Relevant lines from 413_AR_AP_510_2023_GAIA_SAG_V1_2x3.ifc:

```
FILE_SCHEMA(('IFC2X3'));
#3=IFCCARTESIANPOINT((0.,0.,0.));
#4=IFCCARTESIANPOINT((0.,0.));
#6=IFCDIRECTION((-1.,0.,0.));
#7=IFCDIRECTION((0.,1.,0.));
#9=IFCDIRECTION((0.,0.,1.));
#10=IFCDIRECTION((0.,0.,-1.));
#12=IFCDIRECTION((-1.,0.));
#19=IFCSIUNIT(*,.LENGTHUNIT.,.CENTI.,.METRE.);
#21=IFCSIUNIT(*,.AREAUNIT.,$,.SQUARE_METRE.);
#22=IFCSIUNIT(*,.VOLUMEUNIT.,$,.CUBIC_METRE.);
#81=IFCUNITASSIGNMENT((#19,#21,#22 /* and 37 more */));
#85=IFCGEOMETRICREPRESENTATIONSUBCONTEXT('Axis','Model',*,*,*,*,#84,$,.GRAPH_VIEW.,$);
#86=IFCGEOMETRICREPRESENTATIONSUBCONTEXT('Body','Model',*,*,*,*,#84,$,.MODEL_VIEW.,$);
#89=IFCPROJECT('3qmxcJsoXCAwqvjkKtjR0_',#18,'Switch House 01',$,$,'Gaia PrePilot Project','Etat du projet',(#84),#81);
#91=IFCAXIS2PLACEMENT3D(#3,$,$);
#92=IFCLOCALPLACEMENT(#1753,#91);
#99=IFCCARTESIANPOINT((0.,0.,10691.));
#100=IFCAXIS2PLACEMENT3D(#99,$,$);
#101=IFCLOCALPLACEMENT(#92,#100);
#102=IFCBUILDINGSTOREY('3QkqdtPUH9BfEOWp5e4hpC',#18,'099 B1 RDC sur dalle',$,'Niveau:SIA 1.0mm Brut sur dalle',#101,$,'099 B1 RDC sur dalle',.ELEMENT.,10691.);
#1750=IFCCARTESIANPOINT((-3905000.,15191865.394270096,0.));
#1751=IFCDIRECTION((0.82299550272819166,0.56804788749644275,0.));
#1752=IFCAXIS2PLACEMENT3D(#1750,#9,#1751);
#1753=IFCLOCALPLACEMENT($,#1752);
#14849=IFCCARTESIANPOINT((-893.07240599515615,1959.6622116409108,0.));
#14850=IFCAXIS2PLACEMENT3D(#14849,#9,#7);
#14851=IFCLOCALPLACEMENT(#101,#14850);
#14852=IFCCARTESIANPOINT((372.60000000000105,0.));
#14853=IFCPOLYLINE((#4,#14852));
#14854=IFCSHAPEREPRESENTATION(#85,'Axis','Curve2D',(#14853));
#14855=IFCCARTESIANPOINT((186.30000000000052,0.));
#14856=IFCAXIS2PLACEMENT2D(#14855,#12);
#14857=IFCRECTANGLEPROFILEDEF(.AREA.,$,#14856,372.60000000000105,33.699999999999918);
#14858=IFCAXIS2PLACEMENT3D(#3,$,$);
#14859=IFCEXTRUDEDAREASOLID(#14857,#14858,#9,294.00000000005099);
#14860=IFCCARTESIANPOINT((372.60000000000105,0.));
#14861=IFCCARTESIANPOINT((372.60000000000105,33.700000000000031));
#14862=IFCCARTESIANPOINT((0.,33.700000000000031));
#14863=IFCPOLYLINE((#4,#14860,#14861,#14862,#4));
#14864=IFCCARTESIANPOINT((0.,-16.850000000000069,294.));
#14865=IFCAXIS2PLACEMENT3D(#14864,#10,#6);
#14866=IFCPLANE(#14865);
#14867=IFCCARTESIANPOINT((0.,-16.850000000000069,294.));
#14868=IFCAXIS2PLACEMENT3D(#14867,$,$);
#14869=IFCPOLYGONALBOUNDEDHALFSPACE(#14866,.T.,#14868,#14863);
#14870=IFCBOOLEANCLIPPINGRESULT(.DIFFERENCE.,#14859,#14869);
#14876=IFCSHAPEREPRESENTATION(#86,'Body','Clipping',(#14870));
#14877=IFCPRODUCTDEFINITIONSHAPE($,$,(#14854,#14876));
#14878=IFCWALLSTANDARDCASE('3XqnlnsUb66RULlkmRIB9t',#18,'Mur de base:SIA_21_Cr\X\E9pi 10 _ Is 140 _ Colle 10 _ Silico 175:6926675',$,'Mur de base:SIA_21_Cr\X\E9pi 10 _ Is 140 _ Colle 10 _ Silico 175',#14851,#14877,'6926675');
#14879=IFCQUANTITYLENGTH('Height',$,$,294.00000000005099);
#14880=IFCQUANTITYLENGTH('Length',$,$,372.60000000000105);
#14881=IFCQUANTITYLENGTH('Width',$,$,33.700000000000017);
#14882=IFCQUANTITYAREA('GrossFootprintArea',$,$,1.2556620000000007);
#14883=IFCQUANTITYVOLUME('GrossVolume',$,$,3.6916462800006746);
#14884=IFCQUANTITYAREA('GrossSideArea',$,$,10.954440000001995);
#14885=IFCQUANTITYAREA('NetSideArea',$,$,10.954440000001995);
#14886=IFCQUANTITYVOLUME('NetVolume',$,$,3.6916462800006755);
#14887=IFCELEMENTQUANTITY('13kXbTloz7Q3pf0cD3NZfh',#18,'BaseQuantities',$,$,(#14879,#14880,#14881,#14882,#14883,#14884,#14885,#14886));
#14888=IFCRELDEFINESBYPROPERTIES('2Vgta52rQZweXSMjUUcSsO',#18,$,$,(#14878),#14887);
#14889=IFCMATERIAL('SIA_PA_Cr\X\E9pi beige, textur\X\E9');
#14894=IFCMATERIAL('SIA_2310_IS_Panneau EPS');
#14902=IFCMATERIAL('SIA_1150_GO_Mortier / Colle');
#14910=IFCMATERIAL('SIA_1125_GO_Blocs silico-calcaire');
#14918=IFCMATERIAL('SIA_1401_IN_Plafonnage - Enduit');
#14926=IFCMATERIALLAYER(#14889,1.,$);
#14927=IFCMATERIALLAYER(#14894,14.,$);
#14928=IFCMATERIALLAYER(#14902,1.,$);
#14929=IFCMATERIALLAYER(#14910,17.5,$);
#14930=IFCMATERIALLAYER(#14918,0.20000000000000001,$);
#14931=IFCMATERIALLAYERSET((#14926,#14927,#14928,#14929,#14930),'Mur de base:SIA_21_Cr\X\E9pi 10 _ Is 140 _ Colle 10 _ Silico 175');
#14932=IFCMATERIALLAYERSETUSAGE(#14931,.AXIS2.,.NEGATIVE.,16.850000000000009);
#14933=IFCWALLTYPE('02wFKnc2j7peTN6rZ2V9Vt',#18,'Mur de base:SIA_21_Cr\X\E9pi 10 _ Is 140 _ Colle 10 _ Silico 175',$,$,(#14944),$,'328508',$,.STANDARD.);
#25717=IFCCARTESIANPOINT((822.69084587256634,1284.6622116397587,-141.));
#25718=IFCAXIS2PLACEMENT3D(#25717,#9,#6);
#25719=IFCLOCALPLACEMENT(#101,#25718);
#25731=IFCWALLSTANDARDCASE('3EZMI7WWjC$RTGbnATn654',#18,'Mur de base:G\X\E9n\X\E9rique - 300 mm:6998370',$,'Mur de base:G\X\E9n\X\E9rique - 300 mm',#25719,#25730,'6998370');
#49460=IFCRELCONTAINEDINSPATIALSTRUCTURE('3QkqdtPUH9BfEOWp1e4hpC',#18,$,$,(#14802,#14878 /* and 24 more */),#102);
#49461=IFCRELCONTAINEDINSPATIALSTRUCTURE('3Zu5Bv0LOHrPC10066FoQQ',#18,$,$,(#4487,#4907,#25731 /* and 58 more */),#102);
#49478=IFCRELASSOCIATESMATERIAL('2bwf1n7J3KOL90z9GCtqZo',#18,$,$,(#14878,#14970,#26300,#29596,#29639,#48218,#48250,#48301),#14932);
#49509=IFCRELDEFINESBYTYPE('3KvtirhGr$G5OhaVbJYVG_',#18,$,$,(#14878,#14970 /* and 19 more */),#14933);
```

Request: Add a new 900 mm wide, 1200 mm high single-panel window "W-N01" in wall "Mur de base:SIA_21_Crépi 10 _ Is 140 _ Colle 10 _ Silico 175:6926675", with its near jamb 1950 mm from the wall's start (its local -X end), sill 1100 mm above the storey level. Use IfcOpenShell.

```python
import numpy as np
import ifcopenshell
import ifcopenshell.api.feature
import ifcopenshell.api.geometry
import ifcopenshell.api.pset
import ifcopenshell.api.root
import ifcopenshell.api.spatial
import ifcopenshell.api.type
import ifcopenshell.geom
import ifcopenshell.util.element
import ifcopenshell.util.placement
import ifcopenshell.util.representation
import ifcopenshell.util.shape
import ifcopenshell.util.unit

model = ifcopenshell.open("413_AR_AP_510_2023_GAIA_SAG_V1_2x3.ifc")
unit_scale = ifcopenshell.util.unit.calculate_unit_scale(model)
area_scale = ifcopenshell.util.unit.calculate_unit_scale(model, "AREAUNIT")
volume_scale = ifcopenshell.util.unit.calculate_unit_scale(model, "VOLUMEUNIT")
settings = ifcopenshell.geom.settings()


def volume(element):
    """Net volume in cubic metres, openings subtracted."""
    shape = ifcopenshell.geom.create_shape(settings, element)
    return ifcopenshell.util.shape.get_volume(shape.geometry)


wall = model.by_guid("3XqnlnsUb66RULlkmRIB9t")
storey = ifcopenshell.util.element.get_container(wall, ifc_class="IfcBuildingStorey")
context = ifcopenshell.util.representation.get_context(model, "Model", "Body", "MODEL_VIEW")
before = volume(wall)

width, height, from_end, sill = 0.9, 1.2, 1.95, 1.1  # metres

# The wall runs along its own X axis, and the end named is its -X end.
wall_shape = ifcopenshell.geom.create_shape(settings, wall)
x, y, z = ifcopenshell.util.shape.get_vertices(wall_shape.geometry).T
start = x.min() + from_end
face, thickness = float(y.min()), float(y.max() - y.min())
wall_matrix = ifcopenshell.util.placement.get_local_placement(wall.ObjectPlacement)
level = ifcopenshell.util.placement.get_local_placement(storey.ObjectPlacement)[2, 3]


def in_wall(x, y):
    """Placement at x, y metres in the wall's axes, at sill height."""
    matrix = wall_matrix.copy()
    matrix[:, 3] = wall_matrix @ np.array([x / unit_scale, y / unit_scale, 0.0, 1.0])
    matrix[2, 3] = level + sill / unit_scale
    return matrix


# Opening: a box that overshoots both wall faces by 50 mm.
opening = ifcopenshell.api.root.create_entity(model, ifc_class="IfcOpeningElement")
box = ifcopenshell.api.geometry.add_wall_representation(
    model, context=context, length=width, height=height, thickness=thickness + 0.1
)
ifcopenshell.api.geometry.assign_representation(model, product=opening, representation=box)
ifcopenshell.api.geometry.edit_object_placement(model, product=opening, matrix=in_wall(start, face - 0.05), is_si=False)
ifcopenshell.api.feature.add_feature(model, feature=opening, element=wall)

window = ifcopenshell.api.root.create_entity(model, ifc_class="IfcWindow", name="W-N01")
window.OverallWidth, window.OverallHeight = width / unit_scale, height / unit_scale
body = ifcopenshell.api.geometry.add_window_representation(
    model,
    context=context,
    overall_width=window.OverallWidth,
    overall_height=window.OverallHeight,
    partition_type="SINGLE_PANEL",
)
ifcopenshell.api.geometry.assign_representation(model, product=window, representation=body)
ifcopenshell.api.spatial.assign_container(model, products=[window], relating_structure=storey)
fills = ifcopenshell.api.feature.add_filling(model, opening=opening, element=window)
fills.OwnerHistory = window.OwnerHistory  # required in IFC2X3

# IFC2X3 keeps the operation on the window style.
style = ifcopenshell.api.root.create_entity(model, ifc_class="IfcWindowStyle", name="W-N01")
style.OperationType, style.ConstructionType = "SINGLE_PANEL", "NOTDEFINED"
style.ParameterTakesPrecedence = style.Sizeable = False
ifcopenshell.api.type.assign_type(model, related_objects=[window], relating_type=style)

# Centre the window in the wall's thickness.
ifcopenshell.api.geometry.edit_object_placement(model, product=window, matrix=in_wall(start, face), is_si=False)
window_shape = ifcopenshell.geom.create_shape(settings, window)
depth = ifcopenshell.util.shape.get_vertices(window_shape.geometry)[:, 1]
offset = face + thickness / 2 - (depth.min() + depth.max()) / 2
ifcopenshell.api.geometry.edit_object_placement(model, product=window, matrix=in_wall(start, offset), is_si=False)

after = volume(wall)

# Update the wall's stored quantities.
qto = model.by_id(ifcopenshell.util.element.get_pset(wall, "BaseQuantities", should_inherit=False)["id"])
ifcopenshell.api.pset.edit_qto(model, qto=qto, properties={
    "NetSideArea": after / thickness / area_scale,
    "NetVolume": after / volume_scale,
})

print(f"wall volume {before:.3f} -> {after:.3f} m3")

model.write("413_AR_AP_510_2023_GAIA_SAG_V1_2x3_updated.ifc")
```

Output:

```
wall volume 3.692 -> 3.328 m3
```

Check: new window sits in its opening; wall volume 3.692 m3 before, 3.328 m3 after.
